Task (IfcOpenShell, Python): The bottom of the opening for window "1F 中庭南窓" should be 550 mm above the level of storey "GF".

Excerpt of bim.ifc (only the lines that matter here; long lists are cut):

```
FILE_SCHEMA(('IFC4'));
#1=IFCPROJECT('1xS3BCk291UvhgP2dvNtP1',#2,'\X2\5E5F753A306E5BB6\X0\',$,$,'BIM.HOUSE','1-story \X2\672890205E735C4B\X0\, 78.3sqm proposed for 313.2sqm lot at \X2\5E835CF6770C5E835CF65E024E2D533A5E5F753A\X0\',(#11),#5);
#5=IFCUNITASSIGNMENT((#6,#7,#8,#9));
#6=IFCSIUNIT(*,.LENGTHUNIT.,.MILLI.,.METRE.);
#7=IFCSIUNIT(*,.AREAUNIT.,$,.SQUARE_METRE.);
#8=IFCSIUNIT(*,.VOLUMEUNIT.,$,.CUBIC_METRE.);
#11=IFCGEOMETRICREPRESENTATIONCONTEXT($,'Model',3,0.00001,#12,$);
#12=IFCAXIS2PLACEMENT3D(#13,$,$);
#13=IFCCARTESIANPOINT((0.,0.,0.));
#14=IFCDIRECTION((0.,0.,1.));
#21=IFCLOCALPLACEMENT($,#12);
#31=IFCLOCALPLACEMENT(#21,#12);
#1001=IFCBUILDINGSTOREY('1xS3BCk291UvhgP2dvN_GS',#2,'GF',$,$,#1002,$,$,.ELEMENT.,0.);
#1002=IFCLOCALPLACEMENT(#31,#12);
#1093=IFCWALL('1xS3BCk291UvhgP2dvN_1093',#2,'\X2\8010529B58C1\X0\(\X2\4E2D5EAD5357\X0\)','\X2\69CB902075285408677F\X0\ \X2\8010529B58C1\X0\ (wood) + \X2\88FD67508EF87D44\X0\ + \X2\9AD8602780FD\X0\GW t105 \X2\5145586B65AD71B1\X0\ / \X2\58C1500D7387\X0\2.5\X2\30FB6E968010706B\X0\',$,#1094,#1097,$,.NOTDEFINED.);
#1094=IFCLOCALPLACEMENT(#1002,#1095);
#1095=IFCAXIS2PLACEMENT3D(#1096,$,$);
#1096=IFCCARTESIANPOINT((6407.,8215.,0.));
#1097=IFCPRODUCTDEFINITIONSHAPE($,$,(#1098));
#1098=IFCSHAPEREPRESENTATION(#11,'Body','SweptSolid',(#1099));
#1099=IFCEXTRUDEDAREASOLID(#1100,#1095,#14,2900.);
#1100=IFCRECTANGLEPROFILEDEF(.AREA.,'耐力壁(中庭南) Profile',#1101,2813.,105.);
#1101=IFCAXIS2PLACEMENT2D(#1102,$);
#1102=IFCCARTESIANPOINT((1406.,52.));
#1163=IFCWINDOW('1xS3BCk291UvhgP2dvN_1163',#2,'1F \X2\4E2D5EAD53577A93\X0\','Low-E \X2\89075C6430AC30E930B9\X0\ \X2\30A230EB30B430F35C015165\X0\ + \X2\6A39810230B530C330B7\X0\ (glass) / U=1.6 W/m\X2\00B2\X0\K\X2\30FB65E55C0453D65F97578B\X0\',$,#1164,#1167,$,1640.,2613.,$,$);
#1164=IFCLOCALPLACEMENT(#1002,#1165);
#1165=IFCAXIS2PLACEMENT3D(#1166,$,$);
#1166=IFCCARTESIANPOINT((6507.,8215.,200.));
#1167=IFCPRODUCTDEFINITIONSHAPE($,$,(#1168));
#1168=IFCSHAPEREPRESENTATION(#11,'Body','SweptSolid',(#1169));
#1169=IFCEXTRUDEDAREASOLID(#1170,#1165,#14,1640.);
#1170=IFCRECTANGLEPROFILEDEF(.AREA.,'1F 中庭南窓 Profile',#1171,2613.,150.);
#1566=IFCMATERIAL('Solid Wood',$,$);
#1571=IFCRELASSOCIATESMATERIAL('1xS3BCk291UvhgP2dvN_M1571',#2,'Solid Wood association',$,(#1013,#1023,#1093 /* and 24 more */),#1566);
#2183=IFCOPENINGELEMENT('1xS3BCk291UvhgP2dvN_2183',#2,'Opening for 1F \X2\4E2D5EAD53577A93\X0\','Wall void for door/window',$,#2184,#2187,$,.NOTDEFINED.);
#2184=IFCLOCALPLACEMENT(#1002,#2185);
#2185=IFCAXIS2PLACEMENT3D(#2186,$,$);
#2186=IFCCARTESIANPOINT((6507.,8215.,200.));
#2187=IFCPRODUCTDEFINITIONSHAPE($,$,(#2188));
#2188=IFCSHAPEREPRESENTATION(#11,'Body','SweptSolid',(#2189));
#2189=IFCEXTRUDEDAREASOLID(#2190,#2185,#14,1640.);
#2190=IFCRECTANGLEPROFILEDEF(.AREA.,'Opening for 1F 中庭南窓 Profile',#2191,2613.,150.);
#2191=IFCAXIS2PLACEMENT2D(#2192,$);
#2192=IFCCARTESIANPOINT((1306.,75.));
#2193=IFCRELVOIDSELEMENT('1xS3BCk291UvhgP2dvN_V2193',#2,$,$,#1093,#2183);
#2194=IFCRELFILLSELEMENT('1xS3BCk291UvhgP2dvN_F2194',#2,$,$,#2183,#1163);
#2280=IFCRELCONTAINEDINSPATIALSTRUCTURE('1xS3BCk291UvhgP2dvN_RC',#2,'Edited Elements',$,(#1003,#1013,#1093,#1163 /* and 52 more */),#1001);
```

```python
import numpy as np
import ifcopenshell
import ifcopenshell.api.geometry
import ifcopenshell.geom
import ifcopenshell.util.element
import ifcopenshell.util.placement
import ifcopenshell.util.shape
import ifcopenshell.util.unit

model = ifcopenshell.open("bim.ifc")
unit_scale = ifcopenshell.util.unit.calculate_unit_scale(model)

window = model.by_guid("1xS3BCk291UvhgP2dvN_1163")
opening = window.FillsVoids[0].RelatingOpeningElement
storey = ifcopenshell.util.element.get_container(window, ifc_class="IfcBuildingStorey")
level = ifcopenshell.util.placement.get_local_placement(storey.ObjectPlacement)[2, 3]

# The opening's origin need not be at the sill, so measure its lowest point.
shape = ifcopenshell.geom.create_shape(ifcopenshell.geom.settings(), opening)
bottom = ifcopenshell.util.shape.get_shape_bottom_elevation(shape, shape.geometry) / unit_scale
dz = level + 0.55 / unit_scale - bottom

shift = np.array([0.0, 0.0, dz])
# The window is not placed relative to its opening, so move both.
for product in (opening, window):
    matrix = ifcopenshell.util.placement.get_local_placement(product.ObjectPlacement)
    matrix[:3, 3] += shift
    ifcopenshell.api.geometry.edit_object_placement(model, product=product, matrix=matrix, is_si=False)

print(f"moved by {dz * unit_scale:+.3f} m")

model.write("bim_v2.ifc")
```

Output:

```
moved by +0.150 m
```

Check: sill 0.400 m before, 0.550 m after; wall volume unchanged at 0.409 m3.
